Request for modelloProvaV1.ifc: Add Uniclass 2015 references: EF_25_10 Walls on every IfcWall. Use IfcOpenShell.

First a look at what the model holds.

```python
import ifcopenshell

model = ifcopenshell.open("modelloProvaV1.ifc")
print(model.schema)
print("classifications:", [c.Name for c in model.by_type("IfcClassification")])
for ifc_class in ("IfcDoor", "IfcRoof", "IfcStair", "IfcWall", "IfcWindow"):
    print(ifc_class, len(model.by_type(ifc_class)))
```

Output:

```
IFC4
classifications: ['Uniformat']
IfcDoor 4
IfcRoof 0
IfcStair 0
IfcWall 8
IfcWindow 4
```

```python
import ifcopenshell
import ifcopenshell.api.classification

model = ifcopenshell.open("modelloProvaV1.ifc")

system = ifcopenshell.api.classification.add_classification(model, classification="Uniclass 2015")

codes = {
    "IfcWall": ("EF_25_10", "Walls"),
}
for ifc_class, (code, name) in codes.items():
    products = model.by_type(ifc_class)
    ifcopenshell.api.classification.add_reference(
        model, products=products, classification=system, identification=code, name=name
    )
    print(code, len(products))

model.write("modelloProvaV1_v2.ifc")
```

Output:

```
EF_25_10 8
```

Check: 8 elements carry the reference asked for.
